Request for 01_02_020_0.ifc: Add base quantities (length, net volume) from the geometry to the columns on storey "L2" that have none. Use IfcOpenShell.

First a look at what the model holds.

```python
import ifcopenshell
import ifcopenshell.util.element
import ifcopenshell.util.unit

model = ifcopenshell.open("01_02_020_0.ifc")
print(model.schema)
for unit_type in ("LENGTHUNIT", "AREAUNIT", "VOLUMEUNIT"):
    print(unit_type, ifcopenshell.util.unit.calculate_unit_scale(model, unit_type))
storey = next(s for s in model.by_type("IfcBuildingStorey") if s.Name == "L2")
columns = [e for e in ifcopenshell.util.element.get_decomposition(storey) if e.is_a("IfcColumn")]
for e in sorted(columns, key=lambda e: e.id()):
    print(e.id(), e.is_a(), e.Name, list(ifcopenshell.util.element.get_psets(e, qtos_only=True)), sep=" | ")
```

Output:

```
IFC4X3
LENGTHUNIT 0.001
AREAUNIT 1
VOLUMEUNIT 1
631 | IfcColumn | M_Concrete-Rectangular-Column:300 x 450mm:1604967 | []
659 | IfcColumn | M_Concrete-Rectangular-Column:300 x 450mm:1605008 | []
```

```python
import ifcopenshell
import ifcopenshell.api.pset
import ifcopenshell.geom
import ifcopenshell.util.element
import ifcopenshell.util.shape
import ifcopenshell.util.unit

model = ifcopenshell.open("01_02_020_0.ifc")
unit_scale = ifcopenshell.util.unit.calculate_unit_scale(model)
volume_scale = ifcopenshell.util.unit.calculate_unit_scale(model, "VOLUMEUNIT")
settings = ifcopenshell.geom.settings()

storey = next(s for s in model.by_type("IfcBuildingStorey") if s.Name == "L2")
columns = [e for e in ifcopenshell.util.element.get_decomposition(storey) if e.is_a("IfcColumn")]

for e in sorted(columns, key=lambda e: e.id()):
    if ifcopenshell.util.element.get_psets(e, qtos_only=True, should_inherit=False):
        continue
    # Geometry comes back in metres, in the element's own axes.
    shape = ifcopenshell.geom.create_shape(settings, e)
    values = {
        "Length": ifcopenshell.util.shape.get_z(shape.geometry) / unit_scale,
        "NetVolume": ifcopenshell.util.shape.get_volume(shape.geometry) / volume_scale,
    }
    qto = ifcopenshell.api.pset.add_qto(model, product=e, name="Qto_ColumnBaseQuantities")
    ifcopenshell.api.pset.edit_qto(model, qto=qto, properties=values)
    print(e.id(), {k: round(v, 3) for k, v in values.items()})

model.write("01_02_020_0_edited.ifc")
```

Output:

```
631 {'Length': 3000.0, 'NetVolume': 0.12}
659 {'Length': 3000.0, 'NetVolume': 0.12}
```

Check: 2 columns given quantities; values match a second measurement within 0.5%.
